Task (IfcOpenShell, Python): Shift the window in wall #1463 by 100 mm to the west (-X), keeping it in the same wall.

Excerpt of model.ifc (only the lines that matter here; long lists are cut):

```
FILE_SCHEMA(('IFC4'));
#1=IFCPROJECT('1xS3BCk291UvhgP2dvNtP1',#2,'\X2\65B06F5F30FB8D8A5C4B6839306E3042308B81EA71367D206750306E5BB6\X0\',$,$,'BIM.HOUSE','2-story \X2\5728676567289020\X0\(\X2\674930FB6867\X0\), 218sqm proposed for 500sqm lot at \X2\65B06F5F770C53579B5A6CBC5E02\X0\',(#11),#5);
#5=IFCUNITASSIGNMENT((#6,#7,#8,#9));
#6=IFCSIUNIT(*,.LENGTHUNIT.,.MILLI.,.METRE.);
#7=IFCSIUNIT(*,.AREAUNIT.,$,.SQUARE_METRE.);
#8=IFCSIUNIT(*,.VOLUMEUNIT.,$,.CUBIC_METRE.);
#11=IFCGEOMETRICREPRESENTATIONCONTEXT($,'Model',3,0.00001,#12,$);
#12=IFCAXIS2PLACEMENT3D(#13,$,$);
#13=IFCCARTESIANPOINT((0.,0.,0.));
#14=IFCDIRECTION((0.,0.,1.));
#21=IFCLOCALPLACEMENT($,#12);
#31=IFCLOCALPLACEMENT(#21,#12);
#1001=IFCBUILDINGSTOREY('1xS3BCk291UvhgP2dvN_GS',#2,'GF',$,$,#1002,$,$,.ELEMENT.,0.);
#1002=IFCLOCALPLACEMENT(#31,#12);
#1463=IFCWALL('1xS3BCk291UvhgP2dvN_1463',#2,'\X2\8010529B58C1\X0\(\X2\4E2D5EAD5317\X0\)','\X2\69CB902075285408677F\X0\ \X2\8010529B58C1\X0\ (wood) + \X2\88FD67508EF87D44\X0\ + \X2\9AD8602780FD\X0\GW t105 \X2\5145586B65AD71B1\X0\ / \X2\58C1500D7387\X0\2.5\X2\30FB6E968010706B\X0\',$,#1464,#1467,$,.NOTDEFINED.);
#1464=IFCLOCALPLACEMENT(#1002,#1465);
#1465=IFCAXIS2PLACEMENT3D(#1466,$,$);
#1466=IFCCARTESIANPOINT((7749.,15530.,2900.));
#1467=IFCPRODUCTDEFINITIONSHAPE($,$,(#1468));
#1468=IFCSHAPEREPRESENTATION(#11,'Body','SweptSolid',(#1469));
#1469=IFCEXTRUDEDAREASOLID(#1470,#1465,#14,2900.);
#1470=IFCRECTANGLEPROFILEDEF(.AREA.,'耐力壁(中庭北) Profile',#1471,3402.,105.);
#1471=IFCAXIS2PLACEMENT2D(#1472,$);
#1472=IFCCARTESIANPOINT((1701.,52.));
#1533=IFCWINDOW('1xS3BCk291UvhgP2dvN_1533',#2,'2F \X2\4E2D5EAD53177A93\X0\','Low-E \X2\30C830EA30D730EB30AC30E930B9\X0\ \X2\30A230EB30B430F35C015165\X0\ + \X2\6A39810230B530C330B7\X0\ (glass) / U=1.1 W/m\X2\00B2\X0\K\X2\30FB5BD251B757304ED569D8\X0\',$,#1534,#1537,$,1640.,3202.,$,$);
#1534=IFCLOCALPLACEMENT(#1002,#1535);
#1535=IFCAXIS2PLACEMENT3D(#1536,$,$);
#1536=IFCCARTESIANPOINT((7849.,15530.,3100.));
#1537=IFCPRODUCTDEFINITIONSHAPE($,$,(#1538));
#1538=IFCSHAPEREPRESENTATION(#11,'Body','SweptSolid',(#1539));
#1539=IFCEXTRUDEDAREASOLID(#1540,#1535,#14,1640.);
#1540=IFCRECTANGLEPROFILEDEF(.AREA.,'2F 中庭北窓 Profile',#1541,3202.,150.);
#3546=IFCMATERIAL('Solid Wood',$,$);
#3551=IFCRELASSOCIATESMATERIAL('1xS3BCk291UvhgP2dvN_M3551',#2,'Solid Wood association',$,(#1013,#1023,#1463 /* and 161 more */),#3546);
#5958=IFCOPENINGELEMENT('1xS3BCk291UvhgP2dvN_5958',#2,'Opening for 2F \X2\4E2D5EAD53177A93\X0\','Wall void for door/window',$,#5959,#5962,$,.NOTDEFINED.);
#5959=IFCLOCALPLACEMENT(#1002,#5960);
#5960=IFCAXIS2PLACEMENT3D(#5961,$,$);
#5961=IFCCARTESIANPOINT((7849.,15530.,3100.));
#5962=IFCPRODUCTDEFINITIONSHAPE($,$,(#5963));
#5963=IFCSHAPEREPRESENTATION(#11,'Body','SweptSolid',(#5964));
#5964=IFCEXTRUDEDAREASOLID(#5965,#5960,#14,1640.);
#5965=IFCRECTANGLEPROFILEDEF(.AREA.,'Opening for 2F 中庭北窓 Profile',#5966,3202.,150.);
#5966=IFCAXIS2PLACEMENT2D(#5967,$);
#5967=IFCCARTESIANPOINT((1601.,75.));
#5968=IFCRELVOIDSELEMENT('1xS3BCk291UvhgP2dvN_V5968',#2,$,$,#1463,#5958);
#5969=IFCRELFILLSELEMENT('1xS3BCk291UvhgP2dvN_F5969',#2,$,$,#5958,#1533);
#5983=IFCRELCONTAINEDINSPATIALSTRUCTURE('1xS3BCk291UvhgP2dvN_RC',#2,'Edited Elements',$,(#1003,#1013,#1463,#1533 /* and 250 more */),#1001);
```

```python
import ifcopenshell
import ifcopenshell.api.geometry
import ifcopenshell.util.placement

model = ifcopenshell.open("model.ifc")

window = model.by_id(1533)
opening = window.FillsVoids[0].RelatingOpeningElement
wall = opening.VoidsElements[0].RelatingBuildingElement

wall_matrix = ifcopenshell.util.placement.get_local_placement(wall.ObjectPlacement)
shift = wall_matrix[:3, 0] * -100.0
before = ifcopenshell.util.placement.get_local_placement(window.ObjectPlacement)[:3, 3].copy()

# The window is not placed relative to its opening, so move both.
for product in (opening, window):
    matrix = ifcopenshell.util.placement.get_local_placement(product.ObjectPlacement)
    matrix[:3, 3] += shift
    ifcopenshell.api.geometry.edit_object_placement(model, product=product, matrix=matrix, is_si=False)

after = ifcopenshell.util.placement.get_local_placement(window.ObjectPlacement)[:3, 3]
print("window moved by", (after - before).round(3) + 0.0)

model.write("model_edited.ifc")
```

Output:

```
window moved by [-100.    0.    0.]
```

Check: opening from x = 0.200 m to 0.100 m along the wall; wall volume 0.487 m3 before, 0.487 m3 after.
